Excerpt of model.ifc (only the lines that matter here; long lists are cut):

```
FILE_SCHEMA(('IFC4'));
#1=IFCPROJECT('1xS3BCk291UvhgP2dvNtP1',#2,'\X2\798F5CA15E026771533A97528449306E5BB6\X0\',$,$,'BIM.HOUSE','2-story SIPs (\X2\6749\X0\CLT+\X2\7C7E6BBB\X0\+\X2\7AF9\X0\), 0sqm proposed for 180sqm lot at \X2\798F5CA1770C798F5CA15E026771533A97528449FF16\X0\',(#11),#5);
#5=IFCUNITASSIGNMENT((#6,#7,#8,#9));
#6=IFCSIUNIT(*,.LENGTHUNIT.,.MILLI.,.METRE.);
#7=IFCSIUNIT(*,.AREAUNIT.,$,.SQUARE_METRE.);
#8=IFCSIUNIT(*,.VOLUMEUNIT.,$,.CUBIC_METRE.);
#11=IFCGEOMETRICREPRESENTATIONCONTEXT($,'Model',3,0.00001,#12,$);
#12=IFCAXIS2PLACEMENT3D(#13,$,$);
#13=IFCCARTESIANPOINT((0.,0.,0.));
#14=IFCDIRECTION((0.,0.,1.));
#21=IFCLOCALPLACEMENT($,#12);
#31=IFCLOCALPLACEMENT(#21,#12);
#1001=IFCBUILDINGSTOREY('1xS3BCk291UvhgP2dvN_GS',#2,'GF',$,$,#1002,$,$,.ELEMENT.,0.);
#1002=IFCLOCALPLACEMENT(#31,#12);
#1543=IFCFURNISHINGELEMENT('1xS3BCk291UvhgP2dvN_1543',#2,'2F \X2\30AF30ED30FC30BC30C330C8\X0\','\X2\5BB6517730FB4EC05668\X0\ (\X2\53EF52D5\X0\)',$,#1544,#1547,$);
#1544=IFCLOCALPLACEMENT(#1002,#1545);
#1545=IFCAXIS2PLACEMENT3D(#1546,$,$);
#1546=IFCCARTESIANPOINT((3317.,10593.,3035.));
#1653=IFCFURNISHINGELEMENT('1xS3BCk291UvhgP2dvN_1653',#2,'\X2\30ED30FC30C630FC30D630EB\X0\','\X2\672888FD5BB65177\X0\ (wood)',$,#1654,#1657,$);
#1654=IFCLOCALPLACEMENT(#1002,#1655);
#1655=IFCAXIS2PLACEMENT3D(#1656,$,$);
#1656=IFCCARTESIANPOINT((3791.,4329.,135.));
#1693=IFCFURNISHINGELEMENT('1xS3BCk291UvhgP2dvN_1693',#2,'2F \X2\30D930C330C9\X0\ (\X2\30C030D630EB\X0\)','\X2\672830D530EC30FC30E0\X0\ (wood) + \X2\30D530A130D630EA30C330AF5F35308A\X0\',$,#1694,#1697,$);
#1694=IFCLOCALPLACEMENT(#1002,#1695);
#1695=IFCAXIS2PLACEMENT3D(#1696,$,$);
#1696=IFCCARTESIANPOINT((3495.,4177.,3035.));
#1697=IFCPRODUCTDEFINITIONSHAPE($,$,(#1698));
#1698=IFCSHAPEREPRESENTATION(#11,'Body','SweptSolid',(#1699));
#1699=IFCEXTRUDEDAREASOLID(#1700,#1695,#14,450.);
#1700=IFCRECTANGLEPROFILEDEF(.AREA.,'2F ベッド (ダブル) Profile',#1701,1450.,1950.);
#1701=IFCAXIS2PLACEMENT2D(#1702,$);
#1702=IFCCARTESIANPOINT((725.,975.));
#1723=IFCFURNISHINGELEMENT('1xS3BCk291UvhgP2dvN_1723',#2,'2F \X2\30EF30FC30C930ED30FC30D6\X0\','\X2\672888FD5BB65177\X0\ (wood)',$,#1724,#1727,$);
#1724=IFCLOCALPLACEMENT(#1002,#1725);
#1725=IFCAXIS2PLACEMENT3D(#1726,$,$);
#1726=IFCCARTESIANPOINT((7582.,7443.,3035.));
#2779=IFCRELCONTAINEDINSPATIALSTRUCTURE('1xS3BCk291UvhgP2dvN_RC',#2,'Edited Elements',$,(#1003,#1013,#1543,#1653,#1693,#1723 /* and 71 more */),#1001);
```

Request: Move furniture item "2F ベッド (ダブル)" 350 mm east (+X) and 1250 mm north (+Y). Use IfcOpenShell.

```python
import ifcopenshell
import ifcopenshell.api.geometry
import ifcopenshell.util.placement

model = ifcopenshell.open("model.ifc")

item = model.by_guid("1xS3BCk291UvhgP2dvN_1693")
matrix = ifcopenshell.util.placement.get_local_placement(item.ObjectPlacement)
matrix[0, 3] += 350.0
matrix[1, 3] += 1250.0
ifcopenshell.api.geometry.edit_object_placement(model, product=item, matrix=matrix, is_si=False)

print(ifcopenshell.util.placement.get_local_placement(item.ObjectPlacement).round(3) + 0.0)

model.write("model-out.ifc")
```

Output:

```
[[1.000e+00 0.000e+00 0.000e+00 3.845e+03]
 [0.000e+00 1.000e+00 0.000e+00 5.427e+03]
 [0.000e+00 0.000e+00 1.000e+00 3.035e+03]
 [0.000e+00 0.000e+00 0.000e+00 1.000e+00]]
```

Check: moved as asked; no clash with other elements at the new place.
